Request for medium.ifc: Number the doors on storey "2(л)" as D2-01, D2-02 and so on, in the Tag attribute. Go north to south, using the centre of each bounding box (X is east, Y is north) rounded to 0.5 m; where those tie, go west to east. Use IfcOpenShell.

First a look at what the model holds.

```python
import ifcopenshell
import ifcopenshell.util.element
import ifcopenshell.util.placement

model = ifcopenshell.open("medium.ifc")
print(model.schema)
storey = next(s for s in model.by_type("IfcBuildingStorey") if s.Name == "2(л)")
doors = [e for e in ifcopenshell.util.element.get_decomposition(storey) if e.is_a("IfcDoor")]
for e in sorted(doors, key=lambda e: e.id()):
    origin = ifcopenshell.util.placement.get_local_placement(e.ObjectPlacement)[:3, 3]
    print(e.id(), e.Tag, e.Name, origin.round(2) + 0.0, sep=" | ")
```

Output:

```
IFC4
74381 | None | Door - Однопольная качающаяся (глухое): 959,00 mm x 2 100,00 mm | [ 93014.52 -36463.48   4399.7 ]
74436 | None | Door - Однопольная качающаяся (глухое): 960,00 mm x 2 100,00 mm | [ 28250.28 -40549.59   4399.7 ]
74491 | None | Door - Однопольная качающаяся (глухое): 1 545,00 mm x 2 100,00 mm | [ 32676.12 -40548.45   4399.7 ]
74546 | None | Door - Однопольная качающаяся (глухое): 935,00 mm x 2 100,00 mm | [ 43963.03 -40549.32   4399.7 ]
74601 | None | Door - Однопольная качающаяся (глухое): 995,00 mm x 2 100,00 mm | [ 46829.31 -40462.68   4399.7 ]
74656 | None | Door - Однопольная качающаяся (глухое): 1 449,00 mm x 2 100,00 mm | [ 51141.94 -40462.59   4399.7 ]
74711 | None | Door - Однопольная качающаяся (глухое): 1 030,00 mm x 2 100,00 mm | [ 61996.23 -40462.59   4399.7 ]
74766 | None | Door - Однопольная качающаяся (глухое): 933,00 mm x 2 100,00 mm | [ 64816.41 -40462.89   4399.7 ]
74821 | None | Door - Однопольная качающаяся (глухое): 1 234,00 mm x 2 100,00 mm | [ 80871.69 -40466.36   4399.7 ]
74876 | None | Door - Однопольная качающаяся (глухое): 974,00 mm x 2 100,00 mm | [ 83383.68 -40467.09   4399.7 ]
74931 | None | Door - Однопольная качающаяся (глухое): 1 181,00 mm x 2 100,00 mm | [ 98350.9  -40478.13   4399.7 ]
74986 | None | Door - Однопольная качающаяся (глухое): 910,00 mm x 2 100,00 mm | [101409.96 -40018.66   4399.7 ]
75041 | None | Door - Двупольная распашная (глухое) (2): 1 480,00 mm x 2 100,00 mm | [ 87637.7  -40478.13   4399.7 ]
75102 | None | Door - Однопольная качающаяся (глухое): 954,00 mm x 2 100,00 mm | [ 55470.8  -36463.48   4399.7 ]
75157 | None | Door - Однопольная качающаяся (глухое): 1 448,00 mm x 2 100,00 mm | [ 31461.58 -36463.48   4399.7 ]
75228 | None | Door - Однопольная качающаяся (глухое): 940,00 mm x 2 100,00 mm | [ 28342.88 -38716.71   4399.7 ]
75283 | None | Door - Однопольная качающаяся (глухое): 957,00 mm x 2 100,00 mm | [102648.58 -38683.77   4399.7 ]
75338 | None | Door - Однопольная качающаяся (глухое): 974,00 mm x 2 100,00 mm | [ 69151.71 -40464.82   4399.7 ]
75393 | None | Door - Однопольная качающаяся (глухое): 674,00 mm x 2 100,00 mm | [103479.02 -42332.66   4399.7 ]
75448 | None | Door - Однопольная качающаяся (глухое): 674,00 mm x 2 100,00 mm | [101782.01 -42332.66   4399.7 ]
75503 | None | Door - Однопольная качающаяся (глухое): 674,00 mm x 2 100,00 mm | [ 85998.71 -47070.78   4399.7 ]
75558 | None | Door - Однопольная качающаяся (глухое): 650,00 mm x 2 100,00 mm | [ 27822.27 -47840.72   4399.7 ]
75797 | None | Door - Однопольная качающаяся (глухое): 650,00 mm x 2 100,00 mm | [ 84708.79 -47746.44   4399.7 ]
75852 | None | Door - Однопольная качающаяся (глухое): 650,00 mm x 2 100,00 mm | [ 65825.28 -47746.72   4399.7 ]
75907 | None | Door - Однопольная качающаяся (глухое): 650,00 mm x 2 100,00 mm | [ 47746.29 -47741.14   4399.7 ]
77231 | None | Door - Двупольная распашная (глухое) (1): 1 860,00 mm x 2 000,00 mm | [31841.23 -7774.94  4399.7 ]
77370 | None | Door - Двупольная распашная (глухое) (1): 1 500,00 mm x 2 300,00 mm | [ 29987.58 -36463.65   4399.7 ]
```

```python
import ifcopenshell
import ifcopenshell.geom
import ifcopenshell.util.element
import ifcopenshell.util.shape

model = ifcopenshell.open("medium.ifc")
settings = ifcopenshell.geom.settings()
settings.set("use-world-coords", True)


def centre(element):
    shape = ifcopenshell.geom.create_shape(settings, element)
    return ifcopenshell.util.shape.get_bbox_centroid(shape.geometry)


storey = next(s for s in model.by_type("IfcBuildingStorey") if s.Name == "2(л)")
doors = [e for e in ifcopenshell.util.element.get_decomposition(storey) if e.is_a("IfcDoor")]

# Insertion points can sit at a corner or the storey origin, so sort by the geometry (in metres).
centres = {e: centre(e) for e in doors}
doors.sort(key=lambda e: (-round(centres[e][1] / 0.5), centres[e][0]))

for i, e in enumerate(doors, start=1):
    number = f"D2-{i:02d}"
    e.Tag = number
    print(e.id(), number)

model.write("medium_edited.ifc")
```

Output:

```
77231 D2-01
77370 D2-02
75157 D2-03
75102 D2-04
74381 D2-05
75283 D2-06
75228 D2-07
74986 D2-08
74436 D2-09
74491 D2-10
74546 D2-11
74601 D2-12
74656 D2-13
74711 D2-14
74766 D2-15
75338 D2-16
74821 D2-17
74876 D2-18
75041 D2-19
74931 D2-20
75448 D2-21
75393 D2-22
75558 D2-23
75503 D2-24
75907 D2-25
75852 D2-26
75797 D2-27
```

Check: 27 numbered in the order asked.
